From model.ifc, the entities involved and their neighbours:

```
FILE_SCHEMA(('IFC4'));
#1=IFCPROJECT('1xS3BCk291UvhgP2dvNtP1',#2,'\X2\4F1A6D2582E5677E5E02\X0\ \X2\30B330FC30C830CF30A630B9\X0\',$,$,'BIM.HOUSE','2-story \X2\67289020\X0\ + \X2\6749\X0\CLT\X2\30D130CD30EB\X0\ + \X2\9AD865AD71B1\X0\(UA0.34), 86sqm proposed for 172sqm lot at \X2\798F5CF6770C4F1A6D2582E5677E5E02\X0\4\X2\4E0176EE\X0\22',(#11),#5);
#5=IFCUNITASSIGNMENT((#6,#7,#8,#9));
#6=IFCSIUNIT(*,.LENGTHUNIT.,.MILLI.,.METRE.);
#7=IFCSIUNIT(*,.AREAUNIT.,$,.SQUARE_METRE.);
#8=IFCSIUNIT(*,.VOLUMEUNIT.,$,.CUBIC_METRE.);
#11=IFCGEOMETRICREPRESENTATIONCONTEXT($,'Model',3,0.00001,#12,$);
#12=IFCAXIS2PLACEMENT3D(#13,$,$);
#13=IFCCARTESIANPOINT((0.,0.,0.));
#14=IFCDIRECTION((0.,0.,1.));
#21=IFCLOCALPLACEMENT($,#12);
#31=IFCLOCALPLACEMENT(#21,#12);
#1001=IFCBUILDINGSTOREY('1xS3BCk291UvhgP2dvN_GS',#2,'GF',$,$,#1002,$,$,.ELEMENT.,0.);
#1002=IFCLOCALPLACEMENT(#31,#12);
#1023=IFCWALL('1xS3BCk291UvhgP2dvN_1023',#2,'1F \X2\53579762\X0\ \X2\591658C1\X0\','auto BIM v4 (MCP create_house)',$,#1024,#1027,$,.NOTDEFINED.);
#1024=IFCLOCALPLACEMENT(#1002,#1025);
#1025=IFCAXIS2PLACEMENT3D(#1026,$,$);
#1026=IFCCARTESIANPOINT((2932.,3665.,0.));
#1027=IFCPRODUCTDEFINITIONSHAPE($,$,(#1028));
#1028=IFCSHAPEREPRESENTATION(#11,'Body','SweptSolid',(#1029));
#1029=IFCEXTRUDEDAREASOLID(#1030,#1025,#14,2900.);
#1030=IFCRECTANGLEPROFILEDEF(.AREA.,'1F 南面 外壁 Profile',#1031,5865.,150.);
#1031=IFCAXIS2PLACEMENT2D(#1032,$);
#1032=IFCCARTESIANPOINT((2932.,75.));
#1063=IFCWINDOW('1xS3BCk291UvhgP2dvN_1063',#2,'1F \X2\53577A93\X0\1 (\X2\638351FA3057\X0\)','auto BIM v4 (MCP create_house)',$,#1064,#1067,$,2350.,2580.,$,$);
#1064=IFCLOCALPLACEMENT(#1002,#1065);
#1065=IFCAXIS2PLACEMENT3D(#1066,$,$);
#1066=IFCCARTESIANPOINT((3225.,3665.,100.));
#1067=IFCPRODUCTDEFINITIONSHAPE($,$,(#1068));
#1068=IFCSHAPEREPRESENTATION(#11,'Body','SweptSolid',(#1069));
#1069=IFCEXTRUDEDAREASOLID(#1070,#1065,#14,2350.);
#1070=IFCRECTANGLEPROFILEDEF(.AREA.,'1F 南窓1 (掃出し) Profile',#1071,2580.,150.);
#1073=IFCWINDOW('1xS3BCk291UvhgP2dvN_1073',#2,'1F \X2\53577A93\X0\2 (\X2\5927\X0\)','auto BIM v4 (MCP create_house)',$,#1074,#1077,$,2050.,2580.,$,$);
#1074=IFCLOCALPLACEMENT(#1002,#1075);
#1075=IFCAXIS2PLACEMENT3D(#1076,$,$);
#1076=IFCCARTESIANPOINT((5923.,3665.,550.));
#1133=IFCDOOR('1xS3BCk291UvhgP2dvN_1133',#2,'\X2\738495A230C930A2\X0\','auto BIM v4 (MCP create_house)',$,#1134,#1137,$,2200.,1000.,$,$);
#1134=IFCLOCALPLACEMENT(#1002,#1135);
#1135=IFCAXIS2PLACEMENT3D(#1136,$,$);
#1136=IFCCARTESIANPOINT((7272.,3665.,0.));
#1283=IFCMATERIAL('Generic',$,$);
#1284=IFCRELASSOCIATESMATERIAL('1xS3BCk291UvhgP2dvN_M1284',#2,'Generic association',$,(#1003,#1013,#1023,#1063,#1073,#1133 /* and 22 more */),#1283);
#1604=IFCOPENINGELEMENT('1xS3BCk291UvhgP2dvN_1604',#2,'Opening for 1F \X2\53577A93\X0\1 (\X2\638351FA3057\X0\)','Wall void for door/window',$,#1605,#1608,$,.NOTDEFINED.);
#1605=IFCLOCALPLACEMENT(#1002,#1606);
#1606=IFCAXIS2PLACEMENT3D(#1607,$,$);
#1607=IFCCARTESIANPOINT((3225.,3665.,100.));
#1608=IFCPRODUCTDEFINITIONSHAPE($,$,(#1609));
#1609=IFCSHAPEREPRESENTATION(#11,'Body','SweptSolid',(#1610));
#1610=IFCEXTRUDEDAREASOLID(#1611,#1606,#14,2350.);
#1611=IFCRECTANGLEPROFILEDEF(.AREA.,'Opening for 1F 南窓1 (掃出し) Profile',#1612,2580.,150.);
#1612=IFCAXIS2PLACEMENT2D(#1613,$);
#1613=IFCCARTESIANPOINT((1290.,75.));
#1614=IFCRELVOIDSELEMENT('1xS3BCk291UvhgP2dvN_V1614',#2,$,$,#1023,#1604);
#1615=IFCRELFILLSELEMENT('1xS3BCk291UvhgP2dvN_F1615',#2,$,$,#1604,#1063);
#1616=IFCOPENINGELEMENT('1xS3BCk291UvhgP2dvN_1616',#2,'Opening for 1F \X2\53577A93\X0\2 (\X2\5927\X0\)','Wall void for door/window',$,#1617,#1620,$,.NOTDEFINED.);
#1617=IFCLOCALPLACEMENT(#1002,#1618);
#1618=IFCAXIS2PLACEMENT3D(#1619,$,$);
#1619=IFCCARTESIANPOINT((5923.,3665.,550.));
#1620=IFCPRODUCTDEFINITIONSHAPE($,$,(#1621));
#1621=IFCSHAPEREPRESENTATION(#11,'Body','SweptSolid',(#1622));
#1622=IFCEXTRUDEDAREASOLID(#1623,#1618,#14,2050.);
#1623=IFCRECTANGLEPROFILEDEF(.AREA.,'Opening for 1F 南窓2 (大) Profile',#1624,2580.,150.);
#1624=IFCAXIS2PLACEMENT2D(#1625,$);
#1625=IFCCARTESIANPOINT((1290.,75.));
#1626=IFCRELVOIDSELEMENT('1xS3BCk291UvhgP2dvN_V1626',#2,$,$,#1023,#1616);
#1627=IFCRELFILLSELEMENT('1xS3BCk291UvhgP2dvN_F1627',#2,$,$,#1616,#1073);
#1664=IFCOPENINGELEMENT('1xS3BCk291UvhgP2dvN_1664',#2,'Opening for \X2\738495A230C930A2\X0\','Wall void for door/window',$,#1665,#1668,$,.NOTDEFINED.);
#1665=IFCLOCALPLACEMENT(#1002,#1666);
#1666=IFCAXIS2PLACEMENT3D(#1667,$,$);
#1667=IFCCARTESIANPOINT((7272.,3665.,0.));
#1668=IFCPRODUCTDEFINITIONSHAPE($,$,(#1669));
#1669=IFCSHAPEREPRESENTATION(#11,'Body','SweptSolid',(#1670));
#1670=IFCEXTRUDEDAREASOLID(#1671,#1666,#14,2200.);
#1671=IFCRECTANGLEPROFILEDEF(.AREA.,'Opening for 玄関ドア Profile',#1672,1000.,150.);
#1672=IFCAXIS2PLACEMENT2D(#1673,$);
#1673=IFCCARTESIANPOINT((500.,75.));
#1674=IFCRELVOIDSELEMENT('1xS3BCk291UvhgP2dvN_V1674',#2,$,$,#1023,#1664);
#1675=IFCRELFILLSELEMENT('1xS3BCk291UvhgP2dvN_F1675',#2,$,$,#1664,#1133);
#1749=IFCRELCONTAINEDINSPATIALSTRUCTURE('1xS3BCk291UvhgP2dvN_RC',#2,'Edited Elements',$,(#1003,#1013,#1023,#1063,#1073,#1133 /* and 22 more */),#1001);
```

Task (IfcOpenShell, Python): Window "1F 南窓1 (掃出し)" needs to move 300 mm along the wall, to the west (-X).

```python
import ifcopenshell
import ifcopenshell.api.geometry
import ifcopenshell.util.placement
import ifcopenshell.util.unit

model = ifcopenshell.open("model.ifc")
unit_scale = ifcopenshell.util.unit.calculate_unit_scale(model)

window = model.by_guid("1xS3BCk291UvhgP2dvN_1063")
opening = window.FillsVoids[0].RelatingOpeningElement
wall = opening.VoidsElements[0].RelatingBuildingElement

wall_matrix = ifcopenshell.util.placement.get_local_placement(wall.ObjectPlacement)
shift = wall_matrix[:3, 0] * -0.3 / unit_scale
before = ifcopenshell.util.placement.get_local_placement(window.ObjectPlacement)[:3, 3].copy()

# The window is not placed relative to its opening, so move both.
for product in (opening, window):
    matrix = ifcopenshell.util.placement.get_local_placement(product.ObjectPlacement)
    matrix[:3, 3] += shift
    ifcopenshell.api.geometry.edit_object_placement(model, product=product, matrix=matrix, is_si=False)

after = ifcopenshell.util.placement.get_local_placement(window.ObjectPlacement)[:3, 3]
print("window moved by", (after - before).round(3) + 0.0)

model.write("model_rev.ifc")
```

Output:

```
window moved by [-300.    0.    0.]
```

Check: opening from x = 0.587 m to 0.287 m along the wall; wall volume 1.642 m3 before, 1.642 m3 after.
